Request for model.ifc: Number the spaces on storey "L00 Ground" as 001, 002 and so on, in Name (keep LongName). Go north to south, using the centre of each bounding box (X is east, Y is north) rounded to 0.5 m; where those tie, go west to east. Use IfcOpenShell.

First a look at what the model holds.

```python
import ifcopenshell
import ifcopenshell.util.element
import ifcopenshell.util.placement

model = ifcopenshell.open("model.ifc")
print(model.schema)
storey = next(s for s in model.by_type("IfcBuildingStorey") if s.Name == "L00 Ground")
spaces = [e for e in ifcopenshell.util.element.get_decomposition(storey) if e.is_a("IfcSpace")]
for e in sorted(spaces, key=lambda e: e.id()):
    origin = ifcopenshell.util.placement.get_local_placement(e.ObjectPlacement)[:3, 3]
    print(e.id(), e.Name, e.LongName, origin.round(2) + 0.0, sep=" | ")
```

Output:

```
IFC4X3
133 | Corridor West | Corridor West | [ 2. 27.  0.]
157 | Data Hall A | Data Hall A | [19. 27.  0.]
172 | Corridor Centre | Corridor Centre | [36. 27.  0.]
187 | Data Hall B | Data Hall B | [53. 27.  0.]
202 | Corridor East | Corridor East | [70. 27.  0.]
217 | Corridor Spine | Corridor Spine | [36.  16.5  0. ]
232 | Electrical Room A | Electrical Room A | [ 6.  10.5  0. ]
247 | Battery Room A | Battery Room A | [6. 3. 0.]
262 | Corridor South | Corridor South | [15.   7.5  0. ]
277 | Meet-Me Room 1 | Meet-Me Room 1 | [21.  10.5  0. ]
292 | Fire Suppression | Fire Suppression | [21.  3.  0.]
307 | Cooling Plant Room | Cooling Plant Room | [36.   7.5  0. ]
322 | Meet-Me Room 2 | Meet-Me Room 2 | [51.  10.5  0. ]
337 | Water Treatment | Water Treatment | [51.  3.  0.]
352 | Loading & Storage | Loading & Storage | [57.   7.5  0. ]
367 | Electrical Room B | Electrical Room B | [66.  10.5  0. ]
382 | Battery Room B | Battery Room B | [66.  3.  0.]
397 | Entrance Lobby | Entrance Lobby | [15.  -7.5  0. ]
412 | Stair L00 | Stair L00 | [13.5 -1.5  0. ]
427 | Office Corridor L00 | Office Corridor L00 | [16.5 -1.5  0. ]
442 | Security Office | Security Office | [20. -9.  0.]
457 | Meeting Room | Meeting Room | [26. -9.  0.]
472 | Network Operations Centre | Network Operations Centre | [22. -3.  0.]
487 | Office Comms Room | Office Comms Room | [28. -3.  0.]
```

```python
import ifcopenshell
import ifcopenshell.geom
import ifcopenshell.util.element
import ifcopenshell.util.shape

model = ifcopenshell.open("model.ifc")
settings = ifcopenshell.geom.settings()
settings.set("use-world-coords", True)


def centre(element):
    shape = ifcopenshell.geom.create_shape(settings, element)
    return ifcopenshell.util.shape.get_bbox_centroid(shape.geometry)


storey = next(s for s in model.by_type("IfcBuildingStorey") if s.Name == "L00 Ground")
spaces = [e for e in ifcopenshell.util.element.get_decomposition(storey) if e.is_a("IfcSpace")]

# Insertion points can sit at a corner or the storey origin, so sort by the geometry (in metres).
centres = {e: centre(e) for e in spaces}
spaces.sort(key=lambda e: (-round(centres[e][1] / 0.5), centres[e][0]))

for i, e in enumerate(spaces, start=1):
    number = f"0{i:02d}"
    e.Name = number
    print(e.id(), number)

model.write("model_rev.ifc")
```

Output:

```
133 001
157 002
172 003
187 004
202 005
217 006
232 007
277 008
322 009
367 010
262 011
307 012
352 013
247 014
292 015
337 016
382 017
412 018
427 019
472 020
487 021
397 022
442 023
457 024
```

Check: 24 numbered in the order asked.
